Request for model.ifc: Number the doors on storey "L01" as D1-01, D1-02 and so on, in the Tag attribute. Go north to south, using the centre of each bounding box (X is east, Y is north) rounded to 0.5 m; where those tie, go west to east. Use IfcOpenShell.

First a look at what the model holds.

```python
import ifcopenshell
import ifcopenshell.util.element
import ifcopenshell.util.placement

model = ifcopenshell.open("model.ifc")
print(model.schema)
storey = next(s for s in model.by_type("IfcBuildingStorey") if s.Name == "L01")
doors = [e for e in ifcopenshell.util.element.get_decomposition(storey) if e.is_a("IfcDoor")]
for e in sorted(doors, key=lambda e: e.id()):
    origin = ifcopenshell.util.placement.get_local_placement(e.ObjectPlacement)[:3, 3]
    print(e.id(), e.Tag, e.Name, origin.round(2) + 0.0, sep=" | ")
```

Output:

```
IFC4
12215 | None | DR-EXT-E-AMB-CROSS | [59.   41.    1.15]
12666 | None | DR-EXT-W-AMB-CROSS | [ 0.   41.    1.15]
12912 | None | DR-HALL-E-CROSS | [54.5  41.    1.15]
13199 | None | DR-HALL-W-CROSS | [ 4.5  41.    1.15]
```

```python
import ifcopenshell
import ifcopenshell.geom
import ifcopenshell.util.element
import ifcopenshell.util.shape

model = ifcopenshell.open("model.ifc")
settings = ifcopenshell.geom.settings()
settings.set("use-world-coords", True)


def centre(element):
    shape = ifcopenshell.geom.create_shape(settings, element)
    return ifcopenshell.util.shape.get_bbox_centroid(shape.geometry)


storey = next(s for s in model.by_type("IfcBuildingStorey") if s.Name == "L01")
doors = [e for e in ifcopenshell.util.element.get_decomposition(storey) if e.is_a("IfcDoor")]

# Insertion points can sit at a corner or the storey origin, so sort by the geometry (in metres).
centres = {e: centre(e) for e in doors}
doors.sort(key=lambda e: (-round(centres[e][1] / 0.5), centres[e][0]))

for i, e in enumerate(doors, start=1):
    number = f"D1-{i:02d}"
    e.Tag = number
    print(e.id(), number)

model.write("model_updated.ifc")
```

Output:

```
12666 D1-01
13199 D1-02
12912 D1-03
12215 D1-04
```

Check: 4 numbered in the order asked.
